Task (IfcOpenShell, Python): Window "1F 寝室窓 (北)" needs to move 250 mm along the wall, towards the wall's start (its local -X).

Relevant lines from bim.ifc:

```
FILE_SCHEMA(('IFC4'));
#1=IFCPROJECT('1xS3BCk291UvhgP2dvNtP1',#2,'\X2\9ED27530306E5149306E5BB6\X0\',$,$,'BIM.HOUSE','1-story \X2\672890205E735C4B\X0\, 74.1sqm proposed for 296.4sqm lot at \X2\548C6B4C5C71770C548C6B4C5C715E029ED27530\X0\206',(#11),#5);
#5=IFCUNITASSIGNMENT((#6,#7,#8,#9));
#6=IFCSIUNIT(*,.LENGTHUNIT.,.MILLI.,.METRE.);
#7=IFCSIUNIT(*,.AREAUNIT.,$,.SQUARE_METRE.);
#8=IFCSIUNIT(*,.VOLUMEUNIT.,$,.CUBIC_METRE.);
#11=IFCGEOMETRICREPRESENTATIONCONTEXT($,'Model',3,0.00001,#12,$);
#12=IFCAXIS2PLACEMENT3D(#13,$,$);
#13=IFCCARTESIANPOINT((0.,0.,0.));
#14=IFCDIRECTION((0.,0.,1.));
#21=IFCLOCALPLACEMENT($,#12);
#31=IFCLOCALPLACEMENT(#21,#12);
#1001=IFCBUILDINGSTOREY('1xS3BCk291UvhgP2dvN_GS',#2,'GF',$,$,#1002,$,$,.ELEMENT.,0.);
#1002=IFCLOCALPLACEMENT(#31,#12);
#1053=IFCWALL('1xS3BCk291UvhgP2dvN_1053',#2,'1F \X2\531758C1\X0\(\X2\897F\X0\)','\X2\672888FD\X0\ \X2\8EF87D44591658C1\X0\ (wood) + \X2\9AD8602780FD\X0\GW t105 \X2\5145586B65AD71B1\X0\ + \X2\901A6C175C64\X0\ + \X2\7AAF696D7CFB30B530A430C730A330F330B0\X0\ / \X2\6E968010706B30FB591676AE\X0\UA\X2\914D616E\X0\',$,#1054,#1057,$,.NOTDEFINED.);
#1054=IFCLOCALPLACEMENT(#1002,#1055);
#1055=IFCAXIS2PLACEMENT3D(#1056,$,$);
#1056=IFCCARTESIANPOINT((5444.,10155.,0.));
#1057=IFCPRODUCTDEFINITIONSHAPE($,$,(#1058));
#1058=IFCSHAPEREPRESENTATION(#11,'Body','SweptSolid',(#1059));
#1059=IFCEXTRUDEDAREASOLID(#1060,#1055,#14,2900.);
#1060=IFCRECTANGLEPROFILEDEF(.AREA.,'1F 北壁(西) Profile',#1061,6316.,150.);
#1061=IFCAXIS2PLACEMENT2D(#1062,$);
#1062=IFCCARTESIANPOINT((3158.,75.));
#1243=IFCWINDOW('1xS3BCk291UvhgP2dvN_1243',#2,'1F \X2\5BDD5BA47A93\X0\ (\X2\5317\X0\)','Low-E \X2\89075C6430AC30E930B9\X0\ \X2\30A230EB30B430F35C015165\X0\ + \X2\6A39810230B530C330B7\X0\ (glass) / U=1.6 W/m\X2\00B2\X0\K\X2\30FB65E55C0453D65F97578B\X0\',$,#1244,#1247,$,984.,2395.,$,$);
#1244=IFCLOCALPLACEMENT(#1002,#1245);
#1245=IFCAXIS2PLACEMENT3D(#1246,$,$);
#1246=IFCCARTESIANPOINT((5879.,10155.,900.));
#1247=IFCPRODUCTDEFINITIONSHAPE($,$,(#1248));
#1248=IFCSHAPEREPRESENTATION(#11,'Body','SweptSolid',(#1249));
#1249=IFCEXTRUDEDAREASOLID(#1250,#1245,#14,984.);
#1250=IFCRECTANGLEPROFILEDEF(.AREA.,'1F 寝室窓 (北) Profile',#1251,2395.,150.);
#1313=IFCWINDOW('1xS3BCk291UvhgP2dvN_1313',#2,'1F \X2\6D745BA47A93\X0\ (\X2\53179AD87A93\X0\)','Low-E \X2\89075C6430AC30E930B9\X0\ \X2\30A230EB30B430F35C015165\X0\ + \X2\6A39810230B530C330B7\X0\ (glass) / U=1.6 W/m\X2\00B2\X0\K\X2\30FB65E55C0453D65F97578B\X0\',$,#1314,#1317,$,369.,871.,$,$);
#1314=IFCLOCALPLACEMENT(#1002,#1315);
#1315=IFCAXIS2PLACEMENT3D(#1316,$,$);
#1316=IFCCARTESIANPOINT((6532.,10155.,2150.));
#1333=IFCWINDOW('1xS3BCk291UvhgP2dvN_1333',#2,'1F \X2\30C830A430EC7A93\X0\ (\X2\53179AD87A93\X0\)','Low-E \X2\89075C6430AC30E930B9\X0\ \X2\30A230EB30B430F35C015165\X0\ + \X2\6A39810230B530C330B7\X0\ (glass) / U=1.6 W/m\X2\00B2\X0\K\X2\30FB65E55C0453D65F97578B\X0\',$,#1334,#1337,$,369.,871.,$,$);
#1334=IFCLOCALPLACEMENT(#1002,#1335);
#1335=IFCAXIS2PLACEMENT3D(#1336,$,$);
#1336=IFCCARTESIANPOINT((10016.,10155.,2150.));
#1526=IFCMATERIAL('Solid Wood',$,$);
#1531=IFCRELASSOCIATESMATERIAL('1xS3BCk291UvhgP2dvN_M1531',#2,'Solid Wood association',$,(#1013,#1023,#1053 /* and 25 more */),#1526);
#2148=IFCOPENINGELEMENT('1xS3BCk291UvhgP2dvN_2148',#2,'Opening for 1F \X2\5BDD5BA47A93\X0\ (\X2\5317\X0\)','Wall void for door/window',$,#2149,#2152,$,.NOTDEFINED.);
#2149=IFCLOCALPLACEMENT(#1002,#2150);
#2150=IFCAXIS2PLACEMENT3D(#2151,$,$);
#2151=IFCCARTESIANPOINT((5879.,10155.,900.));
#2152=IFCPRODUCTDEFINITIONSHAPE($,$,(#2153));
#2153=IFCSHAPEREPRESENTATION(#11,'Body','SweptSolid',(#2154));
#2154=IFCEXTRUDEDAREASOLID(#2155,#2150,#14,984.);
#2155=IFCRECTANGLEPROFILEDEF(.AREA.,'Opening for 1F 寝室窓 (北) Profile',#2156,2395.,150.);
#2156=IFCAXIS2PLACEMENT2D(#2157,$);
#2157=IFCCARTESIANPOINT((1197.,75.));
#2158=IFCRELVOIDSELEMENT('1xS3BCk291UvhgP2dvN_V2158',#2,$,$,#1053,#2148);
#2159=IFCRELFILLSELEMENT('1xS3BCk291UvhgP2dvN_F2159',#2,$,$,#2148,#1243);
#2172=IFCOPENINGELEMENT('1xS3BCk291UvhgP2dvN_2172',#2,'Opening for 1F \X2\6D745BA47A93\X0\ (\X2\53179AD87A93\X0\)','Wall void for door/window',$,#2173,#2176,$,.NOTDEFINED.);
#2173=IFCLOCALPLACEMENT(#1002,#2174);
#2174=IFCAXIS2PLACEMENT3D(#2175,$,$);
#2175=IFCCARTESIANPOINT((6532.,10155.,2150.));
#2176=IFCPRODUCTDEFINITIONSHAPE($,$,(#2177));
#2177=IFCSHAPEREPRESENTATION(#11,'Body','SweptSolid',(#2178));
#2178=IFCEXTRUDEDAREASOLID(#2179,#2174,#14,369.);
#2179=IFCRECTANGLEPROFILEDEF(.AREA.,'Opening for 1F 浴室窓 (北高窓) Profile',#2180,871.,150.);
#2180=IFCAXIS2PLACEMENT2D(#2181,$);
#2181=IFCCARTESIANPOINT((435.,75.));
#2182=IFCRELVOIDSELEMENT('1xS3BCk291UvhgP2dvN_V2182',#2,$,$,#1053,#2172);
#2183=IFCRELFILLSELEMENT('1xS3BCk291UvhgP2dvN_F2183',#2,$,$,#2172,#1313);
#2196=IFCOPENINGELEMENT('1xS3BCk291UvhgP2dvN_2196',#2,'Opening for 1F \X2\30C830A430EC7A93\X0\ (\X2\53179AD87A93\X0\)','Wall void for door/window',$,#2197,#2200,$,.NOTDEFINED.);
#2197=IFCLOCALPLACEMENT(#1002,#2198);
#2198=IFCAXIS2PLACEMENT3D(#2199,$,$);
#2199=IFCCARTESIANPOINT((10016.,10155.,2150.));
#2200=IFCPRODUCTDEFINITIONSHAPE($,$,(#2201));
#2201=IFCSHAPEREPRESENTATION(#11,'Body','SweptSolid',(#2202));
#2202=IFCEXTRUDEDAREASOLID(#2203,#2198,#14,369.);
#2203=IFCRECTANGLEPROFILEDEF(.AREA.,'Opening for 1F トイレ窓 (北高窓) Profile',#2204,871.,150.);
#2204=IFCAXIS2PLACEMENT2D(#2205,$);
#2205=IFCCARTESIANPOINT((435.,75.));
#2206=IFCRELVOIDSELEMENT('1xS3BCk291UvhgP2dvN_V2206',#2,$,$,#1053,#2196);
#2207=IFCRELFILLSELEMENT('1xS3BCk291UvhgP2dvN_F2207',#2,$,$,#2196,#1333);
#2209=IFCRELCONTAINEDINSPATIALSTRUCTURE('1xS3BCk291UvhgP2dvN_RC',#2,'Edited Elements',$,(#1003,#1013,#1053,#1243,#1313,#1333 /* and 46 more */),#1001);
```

```python
import ifcopenshell
import ifcopenshell.api.geometry
import ifcopenshell.util.placement
import ifcopenshell.util.unit

model = ifcopenshell.open("bim.ifc")
unit_scale = ifcopenshell.util.unit.calculate_unit_scale(model)

window = model.by_guid("1xS3BCk291UvhgP2dvN_1243")
opening = window.FillsVoids[0].RelatingOpeningElement
wall = opening.VoidsElements[0].RelatingBuildingElement

wall_matrix = ifcopenshell.util.placement.get_local_placement(wall.ObjectPlacement)
shift = wall_matrix[:3, 0] * -0.25 / unit_scale
before = ifcopenshell.util.placement.get_local_placement(window.ObjectPlacement)[:3, 3].copy()

# The window is not placed relative to its opening, so move both.
for product in (opening, window):
    matrix = ifcopenshell.util.placement.get_local_placement(product.ObjectPlacement)
    matrix[:3, 3] += shift
    ifcopenshell.api.geometry.edit_object_placement(model, product=product, matrix=matrix, is_si=False)

after = ifcopenshell.util.placement.get_local_placement(window.ObjectPlacement)[:3, 3]
print("window moved by", (after - before).round(3) + 0.0)

model.write("bim_updated.ifc")
```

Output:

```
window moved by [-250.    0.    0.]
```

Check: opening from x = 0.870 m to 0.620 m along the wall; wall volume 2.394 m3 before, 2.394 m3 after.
